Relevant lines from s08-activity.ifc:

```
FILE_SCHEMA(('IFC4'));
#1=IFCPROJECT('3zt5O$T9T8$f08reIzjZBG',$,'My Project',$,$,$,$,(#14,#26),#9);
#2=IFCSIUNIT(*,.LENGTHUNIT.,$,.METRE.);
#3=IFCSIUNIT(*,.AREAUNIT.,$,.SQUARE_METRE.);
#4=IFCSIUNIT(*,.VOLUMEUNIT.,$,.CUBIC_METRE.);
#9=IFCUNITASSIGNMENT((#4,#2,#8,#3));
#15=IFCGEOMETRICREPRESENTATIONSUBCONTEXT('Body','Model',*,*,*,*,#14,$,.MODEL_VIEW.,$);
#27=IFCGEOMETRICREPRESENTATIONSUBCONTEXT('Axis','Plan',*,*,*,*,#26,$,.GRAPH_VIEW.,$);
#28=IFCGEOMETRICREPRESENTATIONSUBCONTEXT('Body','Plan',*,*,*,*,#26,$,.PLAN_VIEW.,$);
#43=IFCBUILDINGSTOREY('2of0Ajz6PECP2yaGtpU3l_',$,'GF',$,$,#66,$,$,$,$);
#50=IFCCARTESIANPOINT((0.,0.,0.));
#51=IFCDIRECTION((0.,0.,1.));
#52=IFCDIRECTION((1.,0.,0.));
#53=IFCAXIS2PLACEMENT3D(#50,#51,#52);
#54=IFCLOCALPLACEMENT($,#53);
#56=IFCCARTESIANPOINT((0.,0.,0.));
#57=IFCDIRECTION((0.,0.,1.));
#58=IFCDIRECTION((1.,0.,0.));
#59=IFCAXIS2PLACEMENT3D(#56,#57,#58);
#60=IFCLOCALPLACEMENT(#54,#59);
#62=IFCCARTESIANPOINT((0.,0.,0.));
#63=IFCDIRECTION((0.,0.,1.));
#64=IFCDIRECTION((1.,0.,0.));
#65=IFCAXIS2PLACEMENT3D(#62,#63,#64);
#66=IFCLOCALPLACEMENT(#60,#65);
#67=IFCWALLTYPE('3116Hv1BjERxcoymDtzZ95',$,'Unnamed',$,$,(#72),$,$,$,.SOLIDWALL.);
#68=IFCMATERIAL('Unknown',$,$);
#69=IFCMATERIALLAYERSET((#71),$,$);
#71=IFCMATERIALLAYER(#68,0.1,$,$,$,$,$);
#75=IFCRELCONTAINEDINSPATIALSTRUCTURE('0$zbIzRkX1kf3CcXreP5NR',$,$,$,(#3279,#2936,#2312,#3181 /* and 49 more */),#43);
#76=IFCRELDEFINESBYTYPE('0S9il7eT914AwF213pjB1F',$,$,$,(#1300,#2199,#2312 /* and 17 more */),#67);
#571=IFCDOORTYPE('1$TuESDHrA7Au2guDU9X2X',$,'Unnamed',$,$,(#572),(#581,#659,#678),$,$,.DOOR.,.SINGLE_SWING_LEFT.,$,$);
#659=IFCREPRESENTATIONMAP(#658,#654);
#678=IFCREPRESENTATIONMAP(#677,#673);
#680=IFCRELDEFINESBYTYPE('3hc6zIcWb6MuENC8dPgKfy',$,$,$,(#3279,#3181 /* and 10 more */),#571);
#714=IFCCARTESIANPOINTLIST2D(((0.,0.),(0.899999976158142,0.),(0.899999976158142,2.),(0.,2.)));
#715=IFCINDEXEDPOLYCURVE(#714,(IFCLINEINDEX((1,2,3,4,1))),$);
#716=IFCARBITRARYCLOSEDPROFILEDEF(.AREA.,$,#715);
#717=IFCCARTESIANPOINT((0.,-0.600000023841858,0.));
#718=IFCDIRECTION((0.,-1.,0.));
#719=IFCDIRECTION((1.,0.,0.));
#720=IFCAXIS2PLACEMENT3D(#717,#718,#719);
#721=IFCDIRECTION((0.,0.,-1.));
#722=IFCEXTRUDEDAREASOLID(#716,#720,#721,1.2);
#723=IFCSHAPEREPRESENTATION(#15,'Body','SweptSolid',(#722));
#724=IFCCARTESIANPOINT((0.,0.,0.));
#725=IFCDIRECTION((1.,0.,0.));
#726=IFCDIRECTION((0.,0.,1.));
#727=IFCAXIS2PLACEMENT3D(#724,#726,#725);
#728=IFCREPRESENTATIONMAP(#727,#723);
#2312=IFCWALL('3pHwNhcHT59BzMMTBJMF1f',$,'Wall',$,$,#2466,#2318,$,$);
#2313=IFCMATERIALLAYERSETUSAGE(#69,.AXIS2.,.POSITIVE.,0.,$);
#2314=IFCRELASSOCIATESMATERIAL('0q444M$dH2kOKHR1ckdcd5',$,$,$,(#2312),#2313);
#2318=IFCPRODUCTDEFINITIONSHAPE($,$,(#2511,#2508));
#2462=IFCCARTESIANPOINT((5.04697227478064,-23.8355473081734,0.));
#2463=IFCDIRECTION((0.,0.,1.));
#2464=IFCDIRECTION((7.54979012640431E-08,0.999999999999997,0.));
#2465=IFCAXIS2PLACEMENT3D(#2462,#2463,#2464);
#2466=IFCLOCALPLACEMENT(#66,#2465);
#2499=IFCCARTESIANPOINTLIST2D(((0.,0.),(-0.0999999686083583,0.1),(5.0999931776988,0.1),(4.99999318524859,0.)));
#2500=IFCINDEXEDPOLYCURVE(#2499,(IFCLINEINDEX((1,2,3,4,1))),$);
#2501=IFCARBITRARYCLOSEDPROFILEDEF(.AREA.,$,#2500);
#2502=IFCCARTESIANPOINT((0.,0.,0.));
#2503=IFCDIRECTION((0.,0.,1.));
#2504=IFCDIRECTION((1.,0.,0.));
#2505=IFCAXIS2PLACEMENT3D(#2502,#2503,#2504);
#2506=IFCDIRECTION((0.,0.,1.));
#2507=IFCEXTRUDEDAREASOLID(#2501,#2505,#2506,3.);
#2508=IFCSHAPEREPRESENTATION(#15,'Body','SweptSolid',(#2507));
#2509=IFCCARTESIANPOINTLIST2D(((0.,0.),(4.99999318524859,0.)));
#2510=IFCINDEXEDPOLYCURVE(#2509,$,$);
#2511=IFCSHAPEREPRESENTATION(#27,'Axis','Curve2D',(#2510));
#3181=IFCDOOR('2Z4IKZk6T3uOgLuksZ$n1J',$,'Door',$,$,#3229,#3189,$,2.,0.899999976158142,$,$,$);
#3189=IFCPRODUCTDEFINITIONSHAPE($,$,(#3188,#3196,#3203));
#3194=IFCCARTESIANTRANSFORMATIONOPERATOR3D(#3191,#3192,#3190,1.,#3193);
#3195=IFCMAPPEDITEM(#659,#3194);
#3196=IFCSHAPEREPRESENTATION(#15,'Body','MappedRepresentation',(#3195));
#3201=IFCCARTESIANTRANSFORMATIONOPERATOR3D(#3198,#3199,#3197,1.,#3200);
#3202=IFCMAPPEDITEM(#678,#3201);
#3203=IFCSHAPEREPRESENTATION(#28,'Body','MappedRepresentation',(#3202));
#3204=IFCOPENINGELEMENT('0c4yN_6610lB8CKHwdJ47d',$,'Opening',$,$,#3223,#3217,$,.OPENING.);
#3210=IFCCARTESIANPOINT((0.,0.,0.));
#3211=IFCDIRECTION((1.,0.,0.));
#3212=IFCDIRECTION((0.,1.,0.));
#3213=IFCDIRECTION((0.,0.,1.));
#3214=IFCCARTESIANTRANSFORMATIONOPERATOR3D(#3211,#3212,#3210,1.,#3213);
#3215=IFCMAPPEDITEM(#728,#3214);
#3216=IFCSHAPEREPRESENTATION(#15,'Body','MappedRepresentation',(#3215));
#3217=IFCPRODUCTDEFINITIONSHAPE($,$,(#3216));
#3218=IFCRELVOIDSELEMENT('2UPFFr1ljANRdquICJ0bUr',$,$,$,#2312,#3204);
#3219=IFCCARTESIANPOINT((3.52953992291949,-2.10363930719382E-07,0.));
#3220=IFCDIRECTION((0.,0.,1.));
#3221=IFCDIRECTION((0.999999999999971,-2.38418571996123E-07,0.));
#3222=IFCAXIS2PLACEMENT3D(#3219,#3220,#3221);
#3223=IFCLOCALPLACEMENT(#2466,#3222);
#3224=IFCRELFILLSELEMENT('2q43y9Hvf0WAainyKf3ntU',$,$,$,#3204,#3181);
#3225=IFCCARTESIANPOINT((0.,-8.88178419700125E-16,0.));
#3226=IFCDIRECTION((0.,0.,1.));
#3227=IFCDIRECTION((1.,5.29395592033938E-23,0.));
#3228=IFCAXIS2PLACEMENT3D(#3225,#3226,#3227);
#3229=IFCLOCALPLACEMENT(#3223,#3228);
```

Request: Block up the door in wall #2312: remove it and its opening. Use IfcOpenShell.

```python
import ifcopenshell
import ifcopenshell.api.feature
import ifcopenshell.api.root
import ifcopenshell.geom
import ifcopenshell.util.shape

model = ifcopenshell.open("s08-activity.ifc")
settings = ifcopenshell.geom.settings()


def volume(element):
    """Net volume in cubic metres, openings subtracted."""
    shape = ifcopenshell.geom.create_shape(settings, element)
    return ifcopenshell.util.shape.get_volume(shape.geometry)


door = model.by_guid("2Z4IKZk6T3uOgLuksZ$n1J")
opening = door.FillsVoids[0].RelatingOpeningElement
wall = opening.VoidsElements[0].RelatingBuildingElement
before = volume(wall)

ifcopenshell.api.root.remove_product(model, product=door)
ifcopenshell.api.feature.remove_feature(model, feature=opening)

after = volume(wall)

print(f"wall volume {before:.3f} -> {after:.3f} m3")

model.write("s08-activity_rev.ifc")
```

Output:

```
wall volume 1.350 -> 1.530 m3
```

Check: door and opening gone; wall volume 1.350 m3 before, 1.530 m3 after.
